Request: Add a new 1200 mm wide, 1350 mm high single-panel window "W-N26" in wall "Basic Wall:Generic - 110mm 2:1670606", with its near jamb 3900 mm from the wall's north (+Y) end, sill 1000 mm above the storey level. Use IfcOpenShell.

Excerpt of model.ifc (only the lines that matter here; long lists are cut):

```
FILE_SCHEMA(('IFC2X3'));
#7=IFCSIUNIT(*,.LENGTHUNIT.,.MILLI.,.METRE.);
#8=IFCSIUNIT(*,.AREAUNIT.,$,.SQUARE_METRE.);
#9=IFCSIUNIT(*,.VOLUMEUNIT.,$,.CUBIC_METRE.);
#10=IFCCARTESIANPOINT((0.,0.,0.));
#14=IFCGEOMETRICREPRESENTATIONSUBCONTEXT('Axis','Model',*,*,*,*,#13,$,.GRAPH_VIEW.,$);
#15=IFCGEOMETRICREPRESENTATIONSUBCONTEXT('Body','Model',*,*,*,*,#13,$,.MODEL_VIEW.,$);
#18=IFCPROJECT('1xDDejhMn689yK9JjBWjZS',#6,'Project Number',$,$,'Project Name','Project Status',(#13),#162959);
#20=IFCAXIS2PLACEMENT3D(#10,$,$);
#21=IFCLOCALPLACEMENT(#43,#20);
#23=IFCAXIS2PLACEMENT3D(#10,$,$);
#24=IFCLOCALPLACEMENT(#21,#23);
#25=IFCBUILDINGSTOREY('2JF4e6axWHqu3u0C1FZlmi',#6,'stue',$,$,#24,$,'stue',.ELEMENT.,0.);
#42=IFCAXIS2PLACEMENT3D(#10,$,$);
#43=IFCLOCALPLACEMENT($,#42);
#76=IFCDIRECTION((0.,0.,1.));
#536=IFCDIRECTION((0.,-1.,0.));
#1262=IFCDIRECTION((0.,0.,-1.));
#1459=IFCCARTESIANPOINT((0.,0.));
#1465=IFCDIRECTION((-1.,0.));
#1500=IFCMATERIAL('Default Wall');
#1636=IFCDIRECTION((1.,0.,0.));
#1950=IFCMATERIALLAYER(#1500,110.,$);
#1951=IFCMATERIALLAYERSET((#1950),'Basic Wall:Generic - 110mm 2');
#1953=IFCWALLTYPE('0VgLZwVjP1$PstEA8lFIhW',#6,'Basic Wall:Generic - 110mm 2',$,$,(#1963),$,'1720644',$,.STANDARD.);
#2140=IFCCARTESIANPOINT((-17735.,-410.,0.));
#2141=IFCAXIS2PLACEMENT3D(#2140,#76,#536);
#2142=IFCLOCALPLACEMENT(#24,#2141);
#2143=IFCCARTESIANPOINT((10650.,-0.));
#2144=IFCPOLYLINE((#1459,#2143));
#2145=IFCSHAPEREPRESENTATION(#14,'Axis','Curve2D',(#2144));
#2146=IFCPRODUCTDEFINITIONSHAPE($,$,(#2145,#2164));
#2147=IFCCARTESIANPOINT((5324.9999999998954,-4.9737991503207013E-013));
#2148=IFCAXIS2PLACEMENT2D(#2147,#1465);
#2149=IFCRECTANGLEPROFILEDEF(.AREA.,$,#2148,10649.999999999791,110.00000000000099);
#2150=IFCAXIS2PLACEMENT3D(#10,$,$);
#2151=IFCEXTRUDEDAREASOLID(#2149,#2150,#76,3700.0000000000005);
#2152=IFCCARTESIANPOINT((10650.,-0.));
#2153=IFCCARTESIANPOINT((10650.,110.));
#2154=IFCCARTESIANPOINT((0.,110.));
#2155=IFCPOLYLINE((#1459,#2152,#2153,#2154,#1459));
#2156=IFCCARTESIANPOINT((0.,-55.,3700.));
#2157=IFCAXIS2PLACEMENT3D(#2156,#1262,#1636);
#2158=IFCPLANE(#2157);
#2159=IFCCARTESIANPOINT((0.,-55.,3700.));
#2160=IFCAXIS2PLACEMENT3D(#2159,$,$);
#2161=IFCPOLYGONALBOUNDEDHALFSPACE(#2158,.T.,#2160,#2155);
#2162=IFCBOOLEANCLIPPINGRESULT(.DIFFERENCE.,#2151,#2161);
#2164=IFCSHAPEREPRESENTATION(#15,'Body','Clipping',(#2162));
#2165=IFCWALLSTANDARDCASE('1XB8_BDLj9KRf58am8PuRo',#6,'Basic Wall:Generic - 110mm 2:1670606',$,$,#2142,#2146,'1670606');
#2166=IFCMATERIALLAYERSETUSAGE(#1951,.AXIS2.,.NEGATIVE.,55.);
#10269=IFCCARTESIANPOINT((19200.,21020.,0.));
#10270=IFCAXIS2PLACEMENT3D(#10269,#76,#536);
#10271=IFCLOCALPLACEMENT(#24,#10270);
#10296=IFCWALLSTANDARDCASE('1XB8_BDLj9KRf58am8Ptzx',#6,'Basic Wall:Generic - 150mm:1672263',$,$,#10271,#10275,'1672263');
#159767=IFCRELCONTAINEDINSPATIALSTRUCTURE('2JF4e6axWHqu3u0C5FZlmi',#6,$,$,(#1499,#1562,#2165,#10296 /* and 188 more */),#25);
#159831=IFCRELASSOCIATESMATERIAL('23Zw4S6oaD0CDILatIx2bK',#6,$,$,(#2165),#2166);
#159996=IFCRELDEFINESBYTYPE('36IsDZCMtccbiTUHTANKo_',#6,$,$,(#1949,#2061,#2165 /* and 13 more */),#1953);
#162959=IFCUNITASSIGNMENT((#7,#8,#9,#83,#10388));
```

```python
import numpy as np
import ifcopenshell
import ifcopenshell.api.feature
import ifcopenshell.api.geometry
import ifcopenshell.api.root
import ifcopenshell.api.spatial
import ifcopenshell.api.type
import ifcopenshell.geom
import ifcopenshell.util.element
import ifcopenshell.util.placement
import ifcopenshell.util.representation
import ifcopenshell.util.shape
import ifcopenshell.util.unit

model = ifcopenshell.open("model.ifc")
unit_scale = ifcopenshell.util.unit.calculate_unit_scale(model)
settings = ifcopenshell.geom.settings()


def volume(element):
    """Net volume in cubic metres, openings subtracted."""
    shape = ifcopenshell.geom.create_shape(settings, element)
    return ifcopenshell.util.shape.get_volume(shape.geometry)


wall = model.by_id(2165)
storey = ifcopenshell.util.element.get_container(wall, ifc_class="IfcBuildingStorey")
context = ifcopenshell.util.representation.get_context(model, "Model", "Body", "MODEL_VIEW")
before = volume(wall)

width, height, from_end, sill = 1.2, 1.35, 3.9, 1  # metres

# The wall runs along its own X axis, and the end named is its -X end.
wall_shape = ifcopenshell.geom.create_shape(settings, wall)
x, y, z = ifcopenshell.util.shape.get_vertices(wall_shape.geometry).T
start = x.min() + from_end
face, thickness = float(y.min()), float(y.max() - y.min())
wall_matrix = ifcopenshell.util.placement.get_local_placement(wall.ObjectPlacement)
level = ifcopenshell.util.placement.get_local_placement(storey.ObjectPlacement)[2, 3]


def in_wall(x, y):
    """Placement at x, y metres in the wall's axes, at sill height."""
    matrix = wall_matrix.copy()
    matrix[:, 3] = wall_matrix @ np.array([x / unit_scale, y / unit_scale, 0.0, 1.0])
    matrix[2, 3] = level + sill / unit_scale
    return matrix


# Opening: a box that overshoots both wall faces by 50 mm.
opening = ifcopenshell.api.root.create_entity(model, ifc_class="IfcOpeningElement")
box = ifcopenshell.api.geometry.add_wall_representation(
    model, context=context, length=width, height=height, thickness=thickness + 0.1
)
ifcopenshell.api.geometry.assign_representation(model, product=opening, representation=box)
ifcopenshell.api.geometry.edit_object_placement(model, product=opening, matrix=in_wall(start, face - 0.05), is_si=False)
ifcopenshell.api.feature.add_feature(model, feature=opening, element=wall)

window = ifcopenshell.api.root.create_entity(model, ifc_class="IfcWindow", name="W-N26")
window.OverallWidth, window.OverallHeight = width / unit_scale, height / unit_scale
body = ifcopenshell.api.geometry.add_window_representation(
    model,
    context=context,
    overall_width=window.OverallWidth,
    overall_height=window.OverallHeight,
    partition_type="SINGLE_PANEL",
)
ifcopenshell.api.geometry.assign_representation(model, product=window, representation=body)
ifcopenshell.api.spatial.assign_container(model, products=[window], relating_structure=storey)
fills = ifcopenshell.api.feature.add_filling(model, opening=opening, element=window)
fills.OwnerHistory = window.OwnerHistory  # required in IFC2X3

# IFC2X3 keeps the operation on the window style.
style = ifcopenshell.api.root.create_entity(model, ifc_class="IfcWindowStyle", name="W-N26")
style.OperationType, style.ConstructionType = "SINGLE_PANEL", "NOTDEFINED"
style.ParameterTakesPrecedence = style.Sizeable = False
ifcopenshell.api.type.assign_type(model, related_objects=[window], relating_type=style)

# Centre the window in the wall's thickness.
ifcopenshell.api.geometry.edit_object_placement(model, product=window, matrix=in_wall(start, face), is_si=False)
window_shape = ifcopenshell.geom.create_shape(settings, window)
depth = ifcopenshell.util.shape.get_vertices(window_shape.geometry)[:, 1]
offset = face + thickness / 2 - (depth.min() + depth.max()) / 2
ifcopenshell.api.geometry.edit_object_placement(model, product=window, matrix=in_wall(start, offset), is_si=False)

after = volume(wall)

print(f"wall volume {before:.3f} -> {after:.3f} m3")

model.write("model_edited.ifc")
```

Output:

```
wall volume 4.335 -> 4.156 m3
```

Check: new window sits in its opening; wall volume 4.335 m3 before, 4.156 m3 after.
